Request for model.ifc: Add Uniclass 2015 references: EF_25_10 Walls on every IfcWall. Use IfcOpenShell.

First a look at what the model holds.

```python
import ifcopenshell

model = ifcopenshell.open("model.ifc")
print(model.schema)
print("classifications:", [c.Name for c in model.by_type("IfcClassification")])
for ifc_class in ("IfcDoor", "IfcRoof", "IfcStair", "IfcWall", "IfcWindow"):
    print(ifc_class, len(model.by_type(ifc_class)))
```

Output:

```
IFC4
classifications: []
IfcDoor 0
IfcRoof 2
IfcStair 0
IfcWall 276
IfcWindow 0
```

```python
import ifcopenshell
import ifcopenshell.api.classification

model = ifcopenshell.open("model.ifc")

system = ifcopenshell.api.classification.add_classification(model, classification="Uniclass 2015")

codes = {
    "IfcWall": ("EF_25_10", "Walls"),
}
for ifc_class, (code, name) in codes.items():
    products = model.by_type(ifc_class)
    ifcopenshell.api.classification.add_reference(
        model, products=products, classification=system, identification=code, name=name
    )
    print(code, len(products))

model.write("model_v2.ifc")
```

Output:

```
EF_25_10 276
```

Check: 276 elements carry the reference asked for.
